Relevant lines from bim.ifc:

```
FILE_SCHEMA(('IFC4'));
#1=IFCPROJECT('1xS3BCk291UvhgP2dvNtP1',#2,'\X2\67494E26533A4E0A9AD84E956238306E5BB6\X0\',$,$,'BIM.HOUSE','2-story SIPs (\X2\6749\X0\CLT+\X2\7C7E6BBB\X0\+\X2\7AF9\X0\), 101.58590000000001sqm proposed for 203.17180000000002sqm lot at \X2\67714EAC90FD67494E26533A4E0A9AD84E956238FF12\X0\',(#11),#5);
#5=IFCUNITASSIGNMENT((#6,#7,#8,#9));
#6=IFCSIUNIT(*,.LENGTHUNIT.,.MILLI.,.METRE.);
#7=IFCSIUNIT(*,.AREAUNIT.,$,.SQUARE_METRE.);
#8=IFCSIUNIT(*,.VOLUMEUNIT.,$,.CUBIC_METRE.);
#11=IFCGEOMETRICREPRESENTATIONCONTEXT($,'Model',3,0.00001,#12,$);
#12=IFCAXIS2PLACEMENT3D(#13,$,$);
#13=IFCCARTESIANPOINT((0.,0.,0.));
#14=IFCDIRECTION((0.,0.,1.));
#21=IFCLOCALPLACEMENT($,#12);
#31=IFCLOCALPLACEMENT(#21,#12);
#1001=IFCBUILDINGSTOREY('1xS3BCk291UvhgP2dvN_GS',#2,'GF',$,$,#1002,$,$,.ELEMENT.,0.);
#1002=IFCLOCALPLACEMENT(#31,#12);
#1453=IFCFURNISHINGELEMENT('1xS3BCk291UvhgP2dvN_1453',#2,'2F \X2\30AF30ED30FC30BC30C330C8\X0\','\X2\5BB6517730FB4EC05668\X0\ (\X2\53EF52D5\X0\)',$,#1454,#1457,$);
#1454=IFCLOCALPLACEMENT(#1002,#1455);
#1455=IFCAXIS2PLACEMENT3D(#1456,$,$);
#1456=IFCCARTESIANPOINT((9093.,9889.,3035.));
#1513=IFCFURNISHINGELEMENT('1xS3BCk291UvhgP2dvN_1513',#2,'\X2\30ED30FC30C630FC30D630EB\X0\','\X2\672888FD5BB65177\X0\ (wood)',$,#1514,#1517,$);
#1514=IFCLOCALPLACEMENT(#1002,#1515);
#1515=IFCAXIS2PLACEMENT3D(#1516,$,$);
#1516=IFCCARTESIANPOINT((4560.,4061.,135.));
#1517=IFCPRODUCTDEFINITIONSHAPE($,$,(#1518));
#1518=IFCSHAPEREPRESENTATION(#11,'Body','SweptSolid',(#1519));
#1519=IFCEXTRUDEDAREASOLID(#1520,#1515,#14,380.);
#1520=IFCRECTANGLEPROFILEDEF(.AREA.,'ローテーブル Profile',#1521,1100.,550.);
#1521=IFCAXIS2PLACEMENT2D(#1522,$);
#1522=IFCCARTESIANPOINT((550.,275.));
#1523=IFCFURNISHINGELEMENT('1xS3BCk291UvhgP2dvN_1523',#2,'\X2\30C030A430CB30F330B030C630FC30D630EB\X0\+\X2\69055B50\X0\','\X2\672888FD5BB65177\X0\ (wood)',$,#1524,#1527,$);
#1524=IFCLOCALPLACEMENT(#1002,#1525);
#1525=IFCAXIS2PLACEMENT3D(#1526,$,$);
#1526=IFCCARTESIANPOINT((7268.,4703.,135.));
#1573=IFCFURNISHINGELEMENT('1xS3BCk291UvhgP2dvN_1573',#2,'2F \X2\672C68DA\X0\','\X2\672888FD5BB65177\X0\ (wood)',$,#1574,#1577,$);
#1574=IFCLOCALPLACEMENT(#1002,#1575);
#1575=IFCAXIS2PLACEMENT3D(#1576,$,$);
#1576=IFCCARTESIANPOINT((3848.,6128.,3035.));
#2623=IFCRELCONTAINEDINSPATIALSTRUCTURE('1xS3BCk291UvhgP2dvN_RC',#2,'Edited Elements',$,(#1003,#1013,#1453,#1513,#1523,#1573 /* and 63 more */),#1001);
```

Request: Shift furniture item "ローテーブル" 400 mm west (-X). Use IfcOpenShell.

```python
import ifcopenshell
import ifcopenshell.api.geometry
import ifcopenshell.util.placement
import ifcopenshell.util.unit

model = ifcopenshell.open("bim.ifc")
unit_scale = ifcopenshell.util.unit.calculate_unit_scale(model)

item = model.by_guid("1xS3BCk291UvhgP2dvN_1513")
matrix = ifcopenshell.util.placement.get_local_placement(item.ObjectPlacement)
matrix[0, 3] -= 0.4 / unit_scale
ifcopenshell.api.geometry.edit_object_placement(model, product=item, matrix=matrix, is_si=False)

print(ifcopenshell.util.placement.get_local_placement(item.ObjectPlacement).round(3) + 0.0)

model.write("bim_edited.ifc")
```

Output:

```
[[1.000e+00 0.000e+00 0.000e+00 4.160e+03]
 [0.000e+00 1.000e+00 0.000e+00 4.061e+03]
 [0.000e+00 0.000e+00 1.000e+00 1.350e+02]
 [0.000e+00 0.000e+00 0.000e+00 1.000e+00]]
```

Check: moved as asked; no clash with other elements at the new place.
